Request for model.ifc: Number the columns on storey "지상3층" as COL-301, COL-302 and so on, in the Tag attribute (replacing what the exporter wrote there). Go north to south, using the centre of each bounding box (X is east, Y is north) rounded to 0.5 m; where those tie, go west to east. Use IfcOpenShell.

First a look at what the model holds.

```python
import ifcopenshell
import ifcopenshell.util.element
import ifcopenshell.util.placement

model = ifcopenshell.open("model.ifc")
print(model.schema)
storey = next(s for s in model.by_type("IfcBuildingStorey") if s.Name == "지상3층")
columns = [e for e in ifcopenshell.util.element.get_decomposition(storey) if e.is_a("IfcColumn")]
for e in sorted(columns, key=lambda e: e.id()):
    origin = ifcopenshell.util.placement.get_local_placement(e.ObjectPlacement)[:3, 3]
    print(e.id(), e.Tag, e.Name, origin.round(2) + 0.0, sep=" | ")
```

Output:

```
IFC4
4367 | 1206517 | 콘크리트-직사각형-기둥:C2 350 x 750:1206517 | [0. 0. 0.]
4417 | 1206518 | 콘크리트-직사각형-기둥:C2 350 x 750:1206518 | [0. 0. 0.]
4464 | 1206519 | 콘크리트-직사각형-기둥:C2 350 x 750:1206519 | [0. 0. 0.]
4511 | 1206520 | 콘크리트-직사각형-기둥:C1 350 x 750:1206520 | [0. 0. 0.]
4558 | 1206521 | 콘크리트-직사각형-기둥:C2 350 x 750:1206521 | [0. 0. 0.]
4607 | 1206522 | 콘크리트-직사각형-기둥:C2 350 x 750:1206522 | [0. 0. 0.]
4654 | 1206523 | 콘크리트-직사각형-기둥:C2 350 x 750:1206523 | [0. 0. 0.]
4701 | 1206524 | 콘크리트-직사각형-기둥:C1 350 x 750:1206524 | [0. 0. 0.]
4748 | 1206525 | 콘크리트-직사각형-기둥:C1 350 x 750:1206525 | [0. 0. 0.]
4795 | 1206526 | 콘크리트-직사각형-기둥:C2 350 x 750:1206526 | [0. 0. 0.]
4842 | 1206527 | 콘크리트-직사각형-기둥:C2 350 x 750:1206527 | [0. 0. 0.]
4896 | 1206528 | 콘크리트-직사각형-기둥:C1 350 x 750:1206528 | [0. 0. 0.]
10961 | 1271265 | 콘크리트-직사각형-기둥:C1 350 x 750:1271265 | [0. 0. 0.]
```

```python
import ifcopenshell
import ifcopenshell.geom
import ifcopenshell.util.element
import ifcopenshell.util.shape

model = ifcopenshell.open("model.ifc")
settings = ifcopenshell.geom.settings()
settings.set("use-world-coords", True)


def centre(element):
    shape = ifcopenshell.geom.create_shape(settings, element)
    return ifcopenshell.util.shape.get_bbox_centroid(shape.geometry)


storey = next(s for s in model.by_type("IfcBuildingStorey") if s.Name == "지상3층")
columns = [e for e in ifcopenshell.util.element.get_decomposition(storey) if e.is_a("IfcColumn")]

# Insertion points can sit at a corner or the storey origin, so sort by the geometry (in metres).
centres = {e: centre(e) for e in columns}
columns.sort(key=lambda e: (-round(centres[e][1] / 0.5), centres[e][0]))

for i, e in enumerate(columns, start=1):
    number = f"COL-3{i:02d}"
    e.Tag = number
    print(e.id(), number)

model.write("model_rev.ifc")
```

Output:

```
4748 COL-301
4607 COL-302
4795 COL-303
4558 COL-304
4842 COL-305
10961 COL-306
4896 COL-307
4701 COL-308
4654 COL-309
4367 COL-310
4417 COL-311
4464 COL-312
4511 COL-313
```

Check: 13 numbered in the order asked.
